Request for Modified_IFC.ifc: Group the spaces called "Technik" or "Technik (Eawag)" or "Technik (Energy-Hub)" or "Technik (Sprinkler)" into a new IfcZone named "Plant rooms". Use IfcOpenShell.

First a look at what the model holds.

```python
import ifcopenshell

model = ifcopenshell.open("Modified_IFC.ifc")
print(model.schema)
seen = {}
for space in model.by_type("IfcSpace"):
    seen[space.LongName] = seen.get(space.LongName, 0) + 1
for name, count in sorted(seen.items(), key=str):
    print(count, "x", name)
print("zones:", [z.Name for z in model.by_type("IfcZone")][:20])
```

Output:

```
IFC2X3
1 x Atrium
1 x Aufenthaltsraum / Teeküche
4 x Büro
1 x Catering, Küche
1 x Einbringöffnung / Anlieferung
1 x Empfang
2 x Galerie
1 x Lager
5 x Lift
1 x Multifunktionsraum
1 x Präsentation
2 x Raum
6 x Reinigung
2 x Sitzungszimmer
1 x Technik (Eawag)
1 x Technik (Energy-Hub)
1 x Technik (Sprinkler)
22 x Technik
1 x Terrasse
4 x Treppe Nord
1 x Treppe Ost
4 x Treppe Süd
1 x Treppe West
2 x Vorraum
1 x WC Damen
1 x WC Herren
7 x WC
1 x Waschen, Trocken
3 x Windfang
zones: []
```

```python
import ifcopenshell
import ifcopenshell.api.group
import ifcopenshell.api.root

model = ifcopenshell.open("Modified_IFC.ifc")

names = {"Technik", "Technik (Eawag)", "Technik (Energy-Hub)", "Technik (Sprinkler)"}
spaces = [s for s in model.by_type("IfcSpace") if s.LongName in names]

zone = ifcopenshell.api.root.create_entity(model, ifc_class="IfcZone", name="Plant rooms")
ifcopenshell.api.group.assign_group(model, products=spaces, group=zone)
print(len(spaces), "spaces in", zone.Name)

model.write("Modified_IFC_edited.ifc")
```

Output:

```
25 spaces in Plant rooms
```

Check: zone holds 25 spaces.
